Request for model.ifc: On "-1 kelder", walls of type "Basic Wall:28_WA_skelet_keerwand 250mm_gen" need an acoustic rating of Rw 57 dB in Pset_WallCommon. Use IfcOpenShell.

First a look at what the model holds.

```python
import ifcopenshell
import ifcopenshell.util.element

model = ifcopenshell.open("model.ifc")
print(model.schema)
storey = next(s for s in model.by_type("IfcBuildingStorey") if s.Name == "-1 kelder")
walls = [e for e in ifcopenshell.util.element.get_decomposition(storey) if e.is_a("IfcWall")]
seen = {}
for e in walls:
    element_type = ifcopenshell.util.element.get_type(e)
    key = (element_type.Name if element_type != e and element_type else None, ifcopenshell.util.element.get_pset(e, "Pset_WallCommon", "AcousticRating"))
    seen[key] = seen.get(key, 0) + 1
for (name, value), count in sorted(seen.items(), key=str):
    print(count, "x", name, "|", value)
```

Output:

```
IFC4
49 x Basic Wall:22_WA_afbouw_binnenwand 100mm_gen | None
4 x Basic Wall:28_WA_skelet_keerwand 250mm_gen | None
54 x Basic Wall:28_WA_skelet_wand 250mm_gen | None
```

```python
import ifcopenshell
import ifcopenshell.api.pset
import ifcopenshell.util.element

model = ifcopenshell.open("model.ifc")

storey = next(s for s in model.by_type("IfcBuildingStorey") if s.Name == "-1 kelder")
walls = [e for e in ifcopenshell.util.element.get_decomposition(storey) if e.is_a("IfcWall")]

count = 0
for e in walls:
    element_type = ifcopenshell.util.element.get_type(e)
    if element_type in (None, e) or element_type.Name != "Basic Wall:28_WA_skelet_keerwand 250mm_gen":
        continue
    # add_pset returns the element's existing set when there is one.
    pset = ifcopenshell.api.pset.add_pset(model, product=e, name="Pset_WallCommon")
    ifcopenshell.api.pset.edit_pset(model, pset=pset, properties={"AcousticRating": "Rw 57 dB"})
    count += 1

print(count, "walls updated")

model.write("model_v2.ifc")
```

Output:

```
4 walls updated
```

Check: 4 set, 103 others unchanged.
